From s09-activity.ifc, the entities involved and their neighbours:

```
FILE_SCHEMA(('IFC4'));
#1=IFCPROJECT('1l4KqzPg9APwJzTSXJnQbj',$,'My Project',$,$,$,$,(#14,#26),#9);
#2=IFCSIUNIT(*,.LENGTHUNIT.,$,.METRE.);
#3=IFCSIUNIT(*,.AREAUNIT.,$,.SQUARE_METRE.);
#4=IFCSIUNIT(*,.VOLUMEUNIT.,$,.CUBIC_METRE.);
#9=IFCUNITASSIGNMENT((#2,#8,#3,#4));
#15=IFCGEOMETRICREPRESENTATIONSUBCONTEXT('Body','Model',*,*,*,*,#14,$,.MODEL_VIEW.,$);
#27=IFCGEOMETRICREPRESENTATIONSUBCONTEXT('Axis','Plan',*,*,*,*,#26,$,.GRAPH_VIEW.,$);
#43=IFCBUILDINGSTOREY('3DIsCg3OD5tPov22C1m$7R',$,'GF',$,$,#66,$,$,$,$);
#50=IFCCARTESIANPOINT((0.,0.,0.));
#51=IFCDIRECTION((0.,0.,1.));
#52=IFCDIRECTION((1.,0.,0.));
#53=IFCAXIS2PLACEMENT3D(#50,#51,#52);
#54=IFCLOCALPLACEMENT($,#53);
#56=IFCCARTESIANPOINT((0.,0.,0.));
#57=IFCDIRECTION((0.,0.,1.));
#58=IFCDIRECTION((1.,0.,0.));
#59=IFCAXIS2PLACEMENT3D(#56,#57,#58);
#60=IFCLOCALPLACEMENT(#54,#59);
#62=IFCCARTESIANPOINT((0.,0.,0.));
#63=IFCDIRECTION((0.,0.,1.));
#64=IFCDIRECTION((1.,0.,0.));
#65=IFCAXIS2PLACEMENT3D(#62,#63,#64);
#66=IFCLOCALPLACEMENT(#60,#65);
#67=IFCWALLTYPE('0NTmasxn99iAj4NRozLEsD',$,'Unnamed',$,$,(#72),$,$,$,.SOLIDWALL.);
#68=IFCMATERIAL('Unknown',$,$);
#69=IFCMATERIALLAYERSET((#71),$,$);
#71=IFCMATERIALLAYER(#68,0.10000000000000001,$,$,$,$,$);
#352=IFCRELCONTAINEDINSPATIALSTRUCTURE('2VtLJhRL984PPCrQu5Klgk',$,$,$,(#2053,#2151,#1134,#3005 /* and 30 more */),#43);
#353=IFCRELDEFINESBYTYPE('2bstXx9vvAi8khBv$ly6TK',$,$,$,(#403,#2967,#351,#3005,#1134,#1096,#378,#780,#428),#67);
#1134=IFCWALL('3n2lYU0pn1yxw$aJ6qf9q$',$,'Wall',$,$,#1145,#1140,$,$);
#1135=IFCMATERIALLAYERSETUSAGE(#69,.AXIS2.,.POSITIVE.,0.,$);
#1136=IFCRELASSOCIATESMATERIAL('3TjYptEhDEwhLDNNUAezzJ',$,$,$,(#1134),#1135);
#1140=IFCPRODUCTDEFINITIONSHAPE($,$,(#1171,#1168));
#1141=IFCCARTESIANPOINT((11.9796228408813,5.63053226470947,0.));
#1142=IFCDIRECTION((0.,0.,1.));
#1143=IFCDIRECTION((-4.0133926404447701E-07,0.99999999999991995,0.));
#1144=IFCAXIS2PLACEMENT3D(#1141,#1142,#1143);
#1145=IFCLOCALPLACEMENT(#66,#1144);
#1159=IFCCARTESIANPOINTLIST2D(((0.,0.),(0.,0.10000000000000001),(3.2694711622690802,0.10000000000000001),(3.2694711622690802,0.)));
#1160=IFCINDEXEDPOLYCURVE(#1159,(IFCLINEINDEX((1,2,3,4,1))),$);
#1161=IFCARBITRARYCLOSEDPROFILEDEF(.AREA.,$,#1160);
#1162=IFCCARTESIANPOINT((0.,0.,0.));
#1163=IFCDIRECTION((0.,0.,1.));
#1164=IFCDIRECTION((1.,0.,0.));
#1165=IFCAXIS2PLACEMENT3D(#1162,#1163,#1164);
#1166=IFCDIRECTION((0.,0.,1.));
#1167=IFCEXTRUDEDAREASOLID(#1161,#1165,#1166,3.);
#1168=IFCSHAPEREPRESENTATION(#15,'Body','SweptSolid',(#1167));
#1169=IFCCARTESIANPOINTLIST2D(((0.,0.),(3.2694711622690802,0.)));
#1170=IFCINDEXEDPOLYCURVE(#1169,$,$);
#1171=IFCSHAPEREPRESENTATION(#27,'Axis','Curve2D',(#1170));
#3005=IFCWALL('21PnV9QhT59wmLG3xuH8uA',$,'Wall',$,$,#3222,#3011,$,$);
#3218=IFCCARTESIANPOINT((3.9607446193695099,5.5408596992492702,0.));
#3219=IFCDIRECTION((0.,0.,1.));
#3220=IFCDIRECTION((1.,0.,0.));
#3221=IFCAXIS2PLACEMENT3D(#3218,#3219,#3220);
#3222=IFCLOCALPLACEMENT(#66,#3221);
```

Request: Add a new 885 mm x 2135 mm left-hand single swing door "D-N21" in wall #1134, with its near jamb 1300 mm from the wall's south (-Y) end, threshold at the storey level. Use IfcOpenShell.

```python
import numpy as np
import ifcopenshell
import ifcopenshell.api.feature
import ifcopenshell.api.geometry
import ifcopenshell.api.root
import ifcopenshell.api.spatial
import ifcopenshell.geom
import ifcopenshell.util.element
import ifcopenshell.util.placement
import ifcopenshell.util.representation
import ifcopenshell.util.shape
import ifcopenshell.util.unit

model = ifcopenshell.open("s09-activity.ifc")
unit_scale = ifcopenshell.util.unit.calculate_unit_scale(model)
settings = ifcopenshell.geom.settings()


def volume(element):
    """Net volume in cubic metres, openings subtracted."""
    shape = ifcopenshell.geom.create_shape(settings, element)
    return ifcopenshell.util.shape.get_volume(shape.geometry)


wall = model.by_id(1134)
storey = ifcopenshell.util.element.get_container(wall, ifc_class="IfcBuildingStorey")
context = ifcopenshell.util.representation.get_context(model, "Model", "Body", "MODEL_VIEW")
before = volume(wall)

width, height, from_end, sill = 0.885, 2.135, 1.3, 0.0  # metres

# The wall runs along its own X axis, and the end named is its -X end.
wall_shape = ifcopenshell.geom.create_shape(settings, wall)
x, y, z = ifcopenshell.util.shape.get_vertices(wall_shape.geometry).T
start = x.min() + from_end
face, thickness = float(y.min()), float(y.max() - y.min())
wall_matrix = ifcopenshell.util.placement.get_local_placement(wall.ObjectPlacement)
level = ifcopenshell.util.placement.get_local_placement(storey.ObjectPlacement)[2, 3]


def in_wall(x, y):
    """Placement at x, y metres in the wall's axes, at sill height."""
    matrix = wall_matrix.copy()
    matrix[:, 3] = wall_matrix @ np.array([x / unit_scale, y / unit_scale, 0.0, 1.0])
    matrix[2, 3] = level + sill / unit_scale
    return matrix


# Opening: a box that overshoots both wall faces by 50 mm.
opening = ifcopenshell.api.root.create_entity(model, ifc_class="IfcOpeningElement", predefined_type="OPENING")
box = ifcopenshell.api.geometry.add_wall_representation(
    model, context=context, length=width, height=height, thickness=thickness + 0.1
)
ifcopenshell.api.geometry.assign_representation(model, product=opening, representation=box)
ifcopenshell.api.geometry.edit_object_placement(model, product=opening, matrix=in_wall(start, face - 0.05), is_si=False)
ifcopenshell.api.feature.add_feature(model, feature=opening, element=wall)

door = ifcopenshell.api.root.create_entity(model, ifc_class="IfcDoor", name="D-N21", predefined_type="DOOR")
door.OverallWidth, door.OverallHeight = width / unit_scale, height / unit_scale
door.OperationType = "SINGLE_SWING_LEFT"
body = ifcopenshell.api.geometry.add_door_representation(
    model,
    context=context,
    overall_width=door.OverallWidth,
    overall_height=door.OverallHeight,
    operation_type="SINGLE_SWING_LEFT",
    lining_properties={"LiningDepth": thickness / unit_scale, "ThresholdDepth": thickness / unit_scale},
)
ifcopenshell.api.geometry.assign_representation(model, product=door, representation=body)
ifcopenshell.api.spatial.assign_container(model, products=[door], relating_structure=storey)
ifcopenshell.api.feature.add_filling(model, opening=opening, element=door)

# The lining spans the wall, so the door starts at the wall face.
ifcopenshell.api.geometry.edit_object_placement(model, product=door, matrix=in_wall(start, face), is_si=False)

after = volume(wall)

print(f"wall volume {before:.3f} -> {after:.3f} m3")

model.write("s09-activity_edited.ifc")
```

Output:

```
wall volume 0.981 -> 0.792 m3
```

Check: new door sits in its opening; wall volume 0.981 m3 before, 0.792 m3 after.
